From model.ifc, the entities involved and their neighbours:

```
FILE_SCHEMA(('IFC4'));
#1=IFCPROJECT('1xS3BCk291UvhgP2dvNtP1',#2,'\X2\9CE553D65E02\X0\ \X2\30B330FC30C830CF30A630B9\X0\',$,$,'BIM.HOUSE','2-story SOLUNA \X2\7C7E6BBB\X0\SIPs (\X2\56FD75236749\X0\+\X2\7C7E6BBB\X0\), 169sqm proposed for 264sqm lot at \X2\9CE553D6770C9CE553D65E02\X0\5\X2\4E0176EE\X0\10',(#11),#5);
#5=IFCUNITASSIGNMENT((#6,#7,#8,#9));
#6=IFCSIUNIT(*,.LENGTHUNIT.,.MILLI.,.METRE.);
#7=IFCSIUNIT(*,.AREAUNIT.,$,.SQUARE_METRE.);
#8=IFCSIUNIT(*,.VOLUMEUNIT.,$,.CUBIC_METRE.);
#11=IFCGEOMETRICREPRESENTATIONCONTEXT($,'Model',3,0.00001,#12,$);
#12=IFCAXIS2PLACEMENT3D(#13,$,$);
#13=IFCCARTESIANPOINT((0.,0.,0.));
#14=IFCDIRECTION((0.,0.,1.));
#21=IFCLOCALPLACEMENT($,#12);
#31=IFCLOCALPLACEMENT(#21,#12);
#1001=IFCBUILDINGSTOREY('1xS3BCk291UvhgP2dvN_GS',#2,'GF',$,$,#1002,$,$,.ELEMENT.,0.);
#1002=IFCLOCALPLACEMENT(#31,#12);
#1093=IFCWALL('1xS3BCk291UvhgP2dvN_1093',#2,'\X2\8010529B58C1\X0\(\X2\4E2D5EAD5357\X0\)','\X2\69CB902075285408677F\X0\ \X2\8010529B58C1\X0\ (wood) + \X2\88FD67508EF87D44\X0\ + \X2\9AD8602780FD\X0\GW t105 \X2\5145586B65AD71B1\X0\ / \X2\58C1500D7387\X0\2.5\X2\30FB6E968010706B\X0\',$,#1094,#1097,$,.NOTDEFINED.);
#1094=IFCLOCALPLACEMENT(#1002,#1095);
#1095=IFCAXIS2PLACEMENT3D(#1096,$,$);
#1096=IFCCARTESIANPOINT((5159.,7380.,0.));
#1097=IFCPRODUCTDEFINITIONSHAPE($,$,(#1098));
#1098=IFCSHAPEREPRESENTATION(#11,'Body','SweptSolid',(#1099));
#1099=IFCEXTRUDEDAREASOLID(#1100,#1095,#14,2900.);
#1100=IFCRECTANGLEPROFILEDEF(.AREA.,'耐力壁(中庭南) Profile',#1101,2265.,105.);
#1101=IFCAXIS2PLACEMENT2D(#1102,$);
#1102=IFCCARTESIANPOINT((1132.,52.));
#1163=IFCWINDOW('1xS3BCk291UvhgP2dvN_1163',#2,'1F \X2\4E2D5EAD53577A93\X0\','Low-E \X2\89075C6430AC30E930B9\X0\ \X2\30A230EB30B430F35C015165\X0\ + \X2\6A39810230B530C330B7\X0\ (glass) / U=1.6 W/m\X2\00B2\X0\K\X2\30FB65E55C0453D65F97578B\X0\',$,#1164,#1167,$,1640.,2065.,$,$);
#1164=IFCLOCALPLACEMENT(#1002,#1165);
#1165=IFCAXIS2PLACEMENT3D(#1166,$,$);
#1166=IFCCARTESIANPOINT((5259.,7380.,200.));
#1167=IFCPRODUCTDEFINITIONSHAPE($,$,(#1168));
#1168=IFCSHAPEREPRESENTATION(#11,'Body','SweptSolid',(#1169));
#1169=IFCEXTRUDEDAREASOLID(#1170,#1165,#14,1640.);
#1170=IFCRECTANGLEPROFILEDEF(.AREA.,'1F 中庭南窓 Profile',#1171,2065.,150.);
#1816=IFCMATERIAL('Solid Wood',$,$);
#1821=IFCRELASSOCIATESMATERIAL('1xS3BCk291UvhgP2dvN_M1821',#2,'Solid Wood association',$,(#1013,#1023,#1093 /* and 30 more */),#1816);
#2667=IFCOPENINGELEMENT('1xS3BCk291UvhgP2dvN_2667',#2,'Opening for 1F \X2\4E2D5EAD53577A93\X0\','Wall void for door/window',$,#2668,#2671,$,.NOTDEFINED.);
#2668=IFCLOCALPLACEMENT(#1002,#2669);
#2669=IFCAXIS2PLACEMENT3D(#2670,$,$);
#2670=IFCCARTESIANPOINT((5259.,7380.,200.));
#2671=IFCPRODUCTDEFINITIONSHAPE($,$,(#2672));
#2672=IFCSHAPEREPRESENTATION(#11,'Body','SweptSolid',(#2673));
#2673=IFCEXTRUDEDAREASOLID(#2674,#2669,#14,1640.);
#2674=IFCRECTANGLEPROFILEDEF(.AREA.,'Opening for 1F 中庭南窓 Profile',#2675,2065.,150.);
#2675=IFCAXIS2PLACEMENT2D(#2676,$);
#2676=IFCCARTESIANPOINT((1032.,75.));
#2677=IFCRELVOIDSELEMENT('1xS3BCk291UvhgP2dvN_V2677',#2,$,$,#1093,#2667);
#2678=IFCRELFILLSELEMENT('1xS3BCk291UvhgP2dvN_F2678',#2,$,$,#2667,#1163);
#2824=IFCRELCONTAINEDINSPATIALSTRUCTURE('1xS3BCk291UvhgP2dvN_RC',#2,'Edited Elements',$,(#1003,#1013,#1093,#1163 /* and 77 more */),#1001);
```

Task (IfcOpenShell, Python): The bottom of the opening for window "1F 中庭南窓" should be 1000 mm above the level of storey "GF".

```python
import numpy as np
import ifcopenshell
import ifcopenshell.api.geometry
import ifcopenshell.geom
import ifcopenshell.util.element
import ifcopenshell.util.placement
import ifcopenshell.util.shape
import ifcopenshell.util.unit

model = ifcopenshell.open("model.ifc")
unit_scale = ifcopenshell.util.unit.calculate_unit_scale(model)

window = model.by_guid("1xS3BCk291UvhgP2dvN_1163")
opening = window.FillsVoids[0].RelatingOpeningElement
storey = ifcopenshell.util.element.get_container(window, ifc_class="IfcBuildingStorey")
level = ifcopenshell.util.placement.get_local_placement(storey.ObjectPlacement)[2, 3]

# The opening's origin need not be at the sill, so measure its lowest point.
shape = ifcopenshell.geom.create_shape(ifcopenshell.geom.settings(), opening)
bottom = ifcopenshell.util.shape.get_shape_bottom_elevation(shape, shape.geometry) / unit_scale
dz = level + 1 / unit_scale - bottom

shift = np.array([0.0, 0.0, dz])
# The window is not placed relative to its opening, so move both.
for product in (opening, window):
    matrix = ifcopenshell.util.placement.get_local_placement(product.ObjectPlacement)
    matrix[:3, 3] += shift
    ifcopenshell.api.geometry.edit_object_placement(model, product=product, matrix=matrix, is_si=False)

print(f"moved by {dz * unit_scale:+.3f} m")

model.write("model-out.ifc")
```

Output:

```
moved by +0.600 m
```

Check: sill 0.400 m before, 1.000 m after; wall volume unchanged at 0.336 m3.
